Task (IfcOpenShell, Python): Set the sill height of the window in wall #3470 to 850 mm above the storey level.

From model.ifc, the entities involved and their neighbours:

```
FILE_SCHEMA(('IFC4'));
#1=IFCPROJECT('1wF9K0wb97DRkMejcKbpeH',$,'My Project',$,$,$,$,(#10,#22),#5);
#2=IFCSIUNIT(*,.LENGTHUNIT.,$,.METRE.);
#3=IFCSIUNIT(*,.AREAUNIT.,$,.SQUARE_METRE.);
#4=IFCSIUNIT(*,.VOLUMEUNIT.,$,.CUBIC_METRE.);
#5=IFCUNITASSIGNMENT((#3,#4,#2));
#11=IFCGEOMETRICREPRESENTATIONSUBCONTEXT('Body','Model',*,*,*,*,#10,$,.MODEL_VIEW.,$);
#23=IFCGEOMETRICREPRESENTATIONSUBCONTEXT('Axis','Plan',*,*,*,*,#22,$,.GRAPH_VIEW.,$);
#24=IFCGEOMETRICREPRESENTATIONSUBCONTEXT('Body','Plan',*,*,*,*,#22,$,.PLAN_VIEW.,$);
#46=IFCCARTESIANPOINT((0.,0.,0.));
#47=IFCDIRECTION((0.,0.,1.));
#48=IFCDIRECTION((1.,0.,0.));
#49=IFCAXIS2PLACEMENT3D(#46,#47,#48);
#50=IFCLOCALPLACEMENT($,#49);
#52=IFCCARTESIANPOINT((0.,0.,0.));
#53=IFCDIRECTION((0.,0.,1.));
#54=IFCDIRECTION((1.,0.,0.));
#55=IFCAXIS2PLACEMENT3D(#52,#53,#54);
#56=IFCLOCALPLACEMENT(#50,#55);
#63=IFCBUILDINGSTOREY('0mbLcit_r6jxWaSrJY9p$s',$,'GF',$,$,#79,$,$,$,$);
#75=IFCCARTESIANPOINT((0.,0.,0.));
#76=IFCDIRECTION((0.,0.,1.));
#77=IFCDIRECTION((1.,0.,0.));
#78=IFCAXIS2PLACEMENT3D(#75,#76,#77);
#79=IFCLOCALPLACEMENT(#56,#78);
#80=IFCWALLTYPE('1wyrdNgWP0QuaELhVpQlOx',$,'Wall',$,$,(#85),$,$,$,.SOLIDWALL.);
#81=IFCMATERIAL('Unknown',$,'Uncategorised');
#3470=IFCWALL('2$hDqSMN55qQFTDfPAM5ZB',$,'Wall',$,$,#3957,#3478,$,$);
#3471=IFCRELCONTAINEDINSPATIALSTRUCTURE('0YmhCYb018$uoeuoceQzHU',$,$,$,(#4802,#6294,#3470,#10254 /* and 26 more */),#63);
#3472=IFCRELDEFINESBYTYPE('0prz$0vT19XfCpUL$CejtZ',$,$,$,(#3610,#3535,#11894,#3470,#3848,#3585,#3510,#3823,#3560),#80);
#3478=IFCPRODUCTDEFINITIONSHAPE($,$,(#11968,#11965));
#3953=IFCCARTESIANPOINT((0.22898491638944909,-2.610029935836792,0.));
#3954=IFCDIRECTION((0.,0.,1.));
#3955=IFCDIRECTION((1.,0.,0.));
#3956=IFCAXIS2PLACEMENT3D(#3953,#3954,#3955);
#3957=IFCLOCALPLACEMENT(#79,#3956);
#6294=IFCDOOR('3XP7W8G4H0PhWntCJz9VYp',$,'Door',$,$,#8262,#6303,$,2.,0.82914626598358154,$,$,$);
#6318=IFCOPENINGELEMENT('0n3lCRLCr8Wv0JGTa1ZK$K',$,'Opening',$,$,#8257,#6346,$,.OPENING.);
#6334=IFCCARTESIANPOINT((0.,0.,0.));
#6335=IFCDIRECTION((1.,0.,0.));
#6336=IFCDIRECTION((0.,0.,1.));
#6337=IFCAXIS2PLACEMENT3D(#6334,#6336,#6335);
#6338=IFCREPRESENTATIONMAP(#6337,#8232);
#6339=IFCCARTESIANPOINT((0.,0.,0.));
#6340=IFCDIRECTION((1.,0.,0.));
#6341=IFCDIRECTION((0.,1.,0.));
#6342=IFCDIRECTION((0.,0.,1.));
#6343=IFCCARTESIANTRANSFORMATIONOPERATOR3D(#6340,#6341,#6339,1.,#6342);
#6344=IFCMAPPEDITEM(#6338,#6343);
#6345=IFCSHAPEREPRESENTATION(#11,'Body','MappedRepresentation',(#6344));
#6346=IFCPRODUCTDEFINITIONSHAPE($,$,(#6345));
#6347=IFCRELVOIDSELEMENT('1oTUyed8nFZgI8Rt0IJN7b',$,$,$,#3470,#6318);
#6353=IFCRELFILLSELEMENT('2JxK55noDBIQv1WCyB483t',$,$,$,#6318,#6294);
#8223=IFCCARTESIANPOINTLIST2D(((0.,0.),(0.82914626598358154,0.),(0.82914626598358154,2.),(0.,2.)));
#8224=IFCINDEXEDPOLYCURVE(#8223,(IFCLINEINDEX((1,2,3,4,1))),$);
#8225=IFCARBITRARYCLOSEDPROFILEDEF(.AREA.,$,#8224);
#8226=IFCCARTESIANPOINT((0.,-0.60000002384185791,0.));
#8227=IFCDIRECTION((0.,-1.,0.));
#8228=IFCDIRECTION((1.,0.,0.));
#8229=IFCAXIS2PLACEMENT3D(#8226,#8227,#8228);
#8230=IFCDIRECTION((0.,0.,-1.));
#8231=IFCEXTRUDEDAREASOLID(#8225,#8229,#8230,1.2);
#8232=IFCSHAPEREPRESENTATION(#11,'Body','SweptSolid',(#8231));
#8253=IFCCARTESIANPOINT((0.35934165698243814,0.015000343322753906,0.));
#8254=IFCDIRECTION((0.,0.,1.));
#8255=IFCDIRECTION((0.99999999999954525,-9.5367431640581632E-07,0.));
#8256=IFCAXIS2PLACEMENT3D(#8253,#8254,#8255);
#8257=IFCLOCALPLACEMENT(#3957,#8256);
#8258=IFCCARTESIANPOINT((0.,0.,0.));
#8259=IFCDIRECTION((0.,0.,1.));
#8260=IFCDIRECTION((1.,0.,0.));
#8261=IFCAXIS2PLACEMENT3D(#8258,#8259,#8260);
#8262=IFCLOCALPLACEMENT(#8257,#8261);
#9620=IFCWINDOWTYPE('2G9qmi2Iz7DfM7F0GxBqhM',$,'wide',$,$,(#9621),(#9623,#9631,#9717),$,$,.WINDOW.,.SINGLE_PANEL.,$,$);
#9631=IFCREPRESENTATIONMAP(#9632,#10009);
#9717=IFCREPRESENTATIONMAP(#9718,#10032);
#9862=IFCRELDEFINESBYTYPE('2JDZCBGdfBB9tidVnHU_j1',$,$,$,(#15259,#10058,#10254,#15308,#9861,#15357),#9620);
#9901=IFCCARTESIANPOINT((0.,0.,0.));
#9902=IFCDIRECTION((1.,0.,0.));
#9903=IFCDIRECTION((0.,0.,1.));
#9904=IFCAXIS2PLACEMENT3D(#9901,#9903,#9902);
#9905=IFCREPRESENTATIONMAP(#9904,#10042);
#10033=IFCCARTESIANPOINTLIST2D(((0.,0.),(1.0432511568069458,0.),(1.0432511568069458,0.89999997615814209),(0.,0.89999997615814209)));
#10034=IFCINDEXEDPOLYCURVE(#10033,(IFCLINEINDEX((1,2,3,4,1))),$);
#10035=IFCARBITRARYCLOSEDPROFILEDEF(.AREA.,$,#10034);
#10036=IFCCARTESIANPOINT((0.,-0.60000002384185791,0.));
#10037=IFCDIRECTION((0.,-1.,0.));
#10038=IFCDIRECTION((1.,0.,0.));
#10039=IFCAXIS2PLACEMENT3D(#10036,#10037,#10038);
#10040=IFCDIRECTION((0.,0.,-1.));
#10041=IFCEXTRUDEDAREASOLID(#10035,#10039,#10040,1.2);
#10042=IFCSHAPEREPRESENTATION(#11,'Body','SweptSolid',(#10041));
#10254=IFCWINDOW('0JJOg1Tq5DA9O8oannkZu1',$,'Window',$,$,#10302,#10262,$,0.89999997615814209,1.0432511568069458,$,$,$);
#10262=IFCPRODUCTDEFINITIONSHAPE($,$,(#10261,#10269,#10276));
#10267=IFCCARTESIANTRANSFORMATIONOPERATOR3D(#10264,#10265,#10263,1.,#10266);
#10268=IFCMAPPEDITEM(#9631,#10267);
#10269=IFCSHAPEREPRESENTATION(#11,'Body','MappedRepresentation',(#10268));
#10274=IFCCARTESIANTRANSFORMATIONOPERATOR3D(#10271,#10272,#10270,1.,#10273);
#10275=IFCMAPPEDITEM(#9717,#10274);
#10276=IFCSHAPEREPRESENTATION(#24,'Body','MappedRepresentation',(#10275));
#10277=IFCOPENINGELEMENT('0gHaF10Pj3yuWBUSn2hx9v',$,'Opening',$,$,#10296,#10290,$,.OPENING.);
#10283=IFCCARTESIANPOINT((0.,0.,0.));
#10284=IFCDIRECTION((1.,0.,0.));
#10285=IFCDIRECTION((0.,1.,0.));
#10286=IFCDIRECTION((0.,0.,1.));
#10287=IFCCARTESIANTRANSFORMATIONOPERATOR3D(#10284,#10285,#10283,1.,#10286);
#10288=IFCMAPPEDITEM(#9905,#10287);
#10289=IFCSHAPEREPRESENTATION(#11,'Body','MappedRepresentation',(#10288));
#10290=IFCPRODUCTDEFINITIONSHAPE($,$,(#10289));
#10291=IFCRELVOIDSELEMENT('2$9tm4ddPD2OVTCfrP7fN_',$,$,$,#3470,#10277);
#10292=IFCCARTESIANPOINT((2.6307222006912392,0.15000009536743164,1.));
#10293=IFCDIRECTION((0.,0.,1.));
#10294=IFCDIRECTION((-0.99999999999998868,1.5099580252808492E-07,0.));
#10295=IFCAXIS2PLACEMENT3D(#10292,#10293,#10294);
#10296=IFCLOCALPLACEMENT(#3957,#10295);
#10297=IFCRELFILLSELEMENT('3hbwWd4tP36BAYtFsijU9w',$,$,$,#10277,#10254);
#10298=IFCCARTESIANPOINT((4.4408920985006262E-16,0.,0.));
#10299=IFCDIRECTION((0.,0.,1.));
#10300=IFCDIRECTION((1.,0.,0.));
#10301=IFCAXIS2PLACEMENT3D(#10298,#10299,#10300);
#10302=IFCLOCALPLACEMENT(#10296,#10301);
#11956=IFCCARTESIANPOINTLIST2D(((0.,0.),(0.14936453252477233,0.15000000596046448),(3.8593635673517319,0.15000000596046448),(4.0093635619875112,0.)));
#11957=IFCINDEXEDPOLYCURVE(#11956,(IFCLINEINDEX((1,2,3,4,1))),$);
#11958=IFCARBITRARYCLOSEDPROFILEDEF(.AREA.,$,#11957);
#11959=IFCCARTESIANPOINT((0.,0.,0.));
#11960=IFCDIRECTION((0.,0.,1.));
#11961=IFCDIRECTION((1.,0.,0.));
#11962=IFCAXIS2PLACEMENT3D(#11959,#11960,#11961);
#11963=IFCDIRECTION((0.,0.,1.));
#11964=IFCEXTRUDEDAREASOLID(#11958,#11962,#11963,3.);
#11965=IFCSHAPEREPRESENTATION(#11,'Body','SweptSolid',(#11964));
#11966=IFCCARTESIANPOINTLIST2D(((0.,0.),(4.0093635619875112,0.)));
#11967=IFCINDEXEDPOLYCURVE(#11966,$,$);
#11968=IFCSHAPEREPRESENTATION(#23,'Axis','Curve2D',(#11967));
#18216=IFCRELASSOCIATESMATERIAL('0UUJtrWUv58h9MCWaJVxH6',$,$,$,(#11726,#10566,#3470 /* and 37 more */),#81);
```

```python
import numpy as np
import ifcopenshell
import ifcopenshell.api.geometry
import ifcopenshell.geom
import ifcopenshell.util.element
import ifcopenshell.util.placement
import ifcopenshell.util.shape
import ifcopenshell.util.unit

model = ifcopenshell.open("model.ifc")
unit_scale = ifcopenshell.util.unit.calculate_unit_scale(model)

window = model.by_guid("0JJOg1Tq5DA9O8oannkZu1")
opening = window.FillsVoids[0].RelatingOpeningElement
storey = ifcopenshell.util.element.get_container(window, ifc_class="IfcBuildingStorey")
level = ifcopenshell.util.placement.get_local_placement(storey.ObjectPlacement)[2, 3]

# The opening's origin need not be at the sill, so measure its lowest point.
shape = ifcopenshell.geom.create_shape(ifcopenshell.geom.settings(), opening)
bottom = ifcopenshell.util.shape.get_shape_bottom_elevation(shape, shape.geometry) / unit_scale
dz = level + 0.85 / unit_scale - bottom

shift = np.array([0.0, 0.0, dz])
# The window is placed relative to its opening, so it follows when the opening moves.
matrix = ifcopenshell.util.placement.get_local_placement(opening.ObjectPlacement)
matrix[:3, 3] += shift
ifcopenshell.api.geometry.edit_object_placement(
    model, product=opening, matrix=matrix, is_si=False, should_transform_children=True
)

print(f"moved by {dz * unit_scale:+.3f} m")

model.write("model_v2.ifc")
```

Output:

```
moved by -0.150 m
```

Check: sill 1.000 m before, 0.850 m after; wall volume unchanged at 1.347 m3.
